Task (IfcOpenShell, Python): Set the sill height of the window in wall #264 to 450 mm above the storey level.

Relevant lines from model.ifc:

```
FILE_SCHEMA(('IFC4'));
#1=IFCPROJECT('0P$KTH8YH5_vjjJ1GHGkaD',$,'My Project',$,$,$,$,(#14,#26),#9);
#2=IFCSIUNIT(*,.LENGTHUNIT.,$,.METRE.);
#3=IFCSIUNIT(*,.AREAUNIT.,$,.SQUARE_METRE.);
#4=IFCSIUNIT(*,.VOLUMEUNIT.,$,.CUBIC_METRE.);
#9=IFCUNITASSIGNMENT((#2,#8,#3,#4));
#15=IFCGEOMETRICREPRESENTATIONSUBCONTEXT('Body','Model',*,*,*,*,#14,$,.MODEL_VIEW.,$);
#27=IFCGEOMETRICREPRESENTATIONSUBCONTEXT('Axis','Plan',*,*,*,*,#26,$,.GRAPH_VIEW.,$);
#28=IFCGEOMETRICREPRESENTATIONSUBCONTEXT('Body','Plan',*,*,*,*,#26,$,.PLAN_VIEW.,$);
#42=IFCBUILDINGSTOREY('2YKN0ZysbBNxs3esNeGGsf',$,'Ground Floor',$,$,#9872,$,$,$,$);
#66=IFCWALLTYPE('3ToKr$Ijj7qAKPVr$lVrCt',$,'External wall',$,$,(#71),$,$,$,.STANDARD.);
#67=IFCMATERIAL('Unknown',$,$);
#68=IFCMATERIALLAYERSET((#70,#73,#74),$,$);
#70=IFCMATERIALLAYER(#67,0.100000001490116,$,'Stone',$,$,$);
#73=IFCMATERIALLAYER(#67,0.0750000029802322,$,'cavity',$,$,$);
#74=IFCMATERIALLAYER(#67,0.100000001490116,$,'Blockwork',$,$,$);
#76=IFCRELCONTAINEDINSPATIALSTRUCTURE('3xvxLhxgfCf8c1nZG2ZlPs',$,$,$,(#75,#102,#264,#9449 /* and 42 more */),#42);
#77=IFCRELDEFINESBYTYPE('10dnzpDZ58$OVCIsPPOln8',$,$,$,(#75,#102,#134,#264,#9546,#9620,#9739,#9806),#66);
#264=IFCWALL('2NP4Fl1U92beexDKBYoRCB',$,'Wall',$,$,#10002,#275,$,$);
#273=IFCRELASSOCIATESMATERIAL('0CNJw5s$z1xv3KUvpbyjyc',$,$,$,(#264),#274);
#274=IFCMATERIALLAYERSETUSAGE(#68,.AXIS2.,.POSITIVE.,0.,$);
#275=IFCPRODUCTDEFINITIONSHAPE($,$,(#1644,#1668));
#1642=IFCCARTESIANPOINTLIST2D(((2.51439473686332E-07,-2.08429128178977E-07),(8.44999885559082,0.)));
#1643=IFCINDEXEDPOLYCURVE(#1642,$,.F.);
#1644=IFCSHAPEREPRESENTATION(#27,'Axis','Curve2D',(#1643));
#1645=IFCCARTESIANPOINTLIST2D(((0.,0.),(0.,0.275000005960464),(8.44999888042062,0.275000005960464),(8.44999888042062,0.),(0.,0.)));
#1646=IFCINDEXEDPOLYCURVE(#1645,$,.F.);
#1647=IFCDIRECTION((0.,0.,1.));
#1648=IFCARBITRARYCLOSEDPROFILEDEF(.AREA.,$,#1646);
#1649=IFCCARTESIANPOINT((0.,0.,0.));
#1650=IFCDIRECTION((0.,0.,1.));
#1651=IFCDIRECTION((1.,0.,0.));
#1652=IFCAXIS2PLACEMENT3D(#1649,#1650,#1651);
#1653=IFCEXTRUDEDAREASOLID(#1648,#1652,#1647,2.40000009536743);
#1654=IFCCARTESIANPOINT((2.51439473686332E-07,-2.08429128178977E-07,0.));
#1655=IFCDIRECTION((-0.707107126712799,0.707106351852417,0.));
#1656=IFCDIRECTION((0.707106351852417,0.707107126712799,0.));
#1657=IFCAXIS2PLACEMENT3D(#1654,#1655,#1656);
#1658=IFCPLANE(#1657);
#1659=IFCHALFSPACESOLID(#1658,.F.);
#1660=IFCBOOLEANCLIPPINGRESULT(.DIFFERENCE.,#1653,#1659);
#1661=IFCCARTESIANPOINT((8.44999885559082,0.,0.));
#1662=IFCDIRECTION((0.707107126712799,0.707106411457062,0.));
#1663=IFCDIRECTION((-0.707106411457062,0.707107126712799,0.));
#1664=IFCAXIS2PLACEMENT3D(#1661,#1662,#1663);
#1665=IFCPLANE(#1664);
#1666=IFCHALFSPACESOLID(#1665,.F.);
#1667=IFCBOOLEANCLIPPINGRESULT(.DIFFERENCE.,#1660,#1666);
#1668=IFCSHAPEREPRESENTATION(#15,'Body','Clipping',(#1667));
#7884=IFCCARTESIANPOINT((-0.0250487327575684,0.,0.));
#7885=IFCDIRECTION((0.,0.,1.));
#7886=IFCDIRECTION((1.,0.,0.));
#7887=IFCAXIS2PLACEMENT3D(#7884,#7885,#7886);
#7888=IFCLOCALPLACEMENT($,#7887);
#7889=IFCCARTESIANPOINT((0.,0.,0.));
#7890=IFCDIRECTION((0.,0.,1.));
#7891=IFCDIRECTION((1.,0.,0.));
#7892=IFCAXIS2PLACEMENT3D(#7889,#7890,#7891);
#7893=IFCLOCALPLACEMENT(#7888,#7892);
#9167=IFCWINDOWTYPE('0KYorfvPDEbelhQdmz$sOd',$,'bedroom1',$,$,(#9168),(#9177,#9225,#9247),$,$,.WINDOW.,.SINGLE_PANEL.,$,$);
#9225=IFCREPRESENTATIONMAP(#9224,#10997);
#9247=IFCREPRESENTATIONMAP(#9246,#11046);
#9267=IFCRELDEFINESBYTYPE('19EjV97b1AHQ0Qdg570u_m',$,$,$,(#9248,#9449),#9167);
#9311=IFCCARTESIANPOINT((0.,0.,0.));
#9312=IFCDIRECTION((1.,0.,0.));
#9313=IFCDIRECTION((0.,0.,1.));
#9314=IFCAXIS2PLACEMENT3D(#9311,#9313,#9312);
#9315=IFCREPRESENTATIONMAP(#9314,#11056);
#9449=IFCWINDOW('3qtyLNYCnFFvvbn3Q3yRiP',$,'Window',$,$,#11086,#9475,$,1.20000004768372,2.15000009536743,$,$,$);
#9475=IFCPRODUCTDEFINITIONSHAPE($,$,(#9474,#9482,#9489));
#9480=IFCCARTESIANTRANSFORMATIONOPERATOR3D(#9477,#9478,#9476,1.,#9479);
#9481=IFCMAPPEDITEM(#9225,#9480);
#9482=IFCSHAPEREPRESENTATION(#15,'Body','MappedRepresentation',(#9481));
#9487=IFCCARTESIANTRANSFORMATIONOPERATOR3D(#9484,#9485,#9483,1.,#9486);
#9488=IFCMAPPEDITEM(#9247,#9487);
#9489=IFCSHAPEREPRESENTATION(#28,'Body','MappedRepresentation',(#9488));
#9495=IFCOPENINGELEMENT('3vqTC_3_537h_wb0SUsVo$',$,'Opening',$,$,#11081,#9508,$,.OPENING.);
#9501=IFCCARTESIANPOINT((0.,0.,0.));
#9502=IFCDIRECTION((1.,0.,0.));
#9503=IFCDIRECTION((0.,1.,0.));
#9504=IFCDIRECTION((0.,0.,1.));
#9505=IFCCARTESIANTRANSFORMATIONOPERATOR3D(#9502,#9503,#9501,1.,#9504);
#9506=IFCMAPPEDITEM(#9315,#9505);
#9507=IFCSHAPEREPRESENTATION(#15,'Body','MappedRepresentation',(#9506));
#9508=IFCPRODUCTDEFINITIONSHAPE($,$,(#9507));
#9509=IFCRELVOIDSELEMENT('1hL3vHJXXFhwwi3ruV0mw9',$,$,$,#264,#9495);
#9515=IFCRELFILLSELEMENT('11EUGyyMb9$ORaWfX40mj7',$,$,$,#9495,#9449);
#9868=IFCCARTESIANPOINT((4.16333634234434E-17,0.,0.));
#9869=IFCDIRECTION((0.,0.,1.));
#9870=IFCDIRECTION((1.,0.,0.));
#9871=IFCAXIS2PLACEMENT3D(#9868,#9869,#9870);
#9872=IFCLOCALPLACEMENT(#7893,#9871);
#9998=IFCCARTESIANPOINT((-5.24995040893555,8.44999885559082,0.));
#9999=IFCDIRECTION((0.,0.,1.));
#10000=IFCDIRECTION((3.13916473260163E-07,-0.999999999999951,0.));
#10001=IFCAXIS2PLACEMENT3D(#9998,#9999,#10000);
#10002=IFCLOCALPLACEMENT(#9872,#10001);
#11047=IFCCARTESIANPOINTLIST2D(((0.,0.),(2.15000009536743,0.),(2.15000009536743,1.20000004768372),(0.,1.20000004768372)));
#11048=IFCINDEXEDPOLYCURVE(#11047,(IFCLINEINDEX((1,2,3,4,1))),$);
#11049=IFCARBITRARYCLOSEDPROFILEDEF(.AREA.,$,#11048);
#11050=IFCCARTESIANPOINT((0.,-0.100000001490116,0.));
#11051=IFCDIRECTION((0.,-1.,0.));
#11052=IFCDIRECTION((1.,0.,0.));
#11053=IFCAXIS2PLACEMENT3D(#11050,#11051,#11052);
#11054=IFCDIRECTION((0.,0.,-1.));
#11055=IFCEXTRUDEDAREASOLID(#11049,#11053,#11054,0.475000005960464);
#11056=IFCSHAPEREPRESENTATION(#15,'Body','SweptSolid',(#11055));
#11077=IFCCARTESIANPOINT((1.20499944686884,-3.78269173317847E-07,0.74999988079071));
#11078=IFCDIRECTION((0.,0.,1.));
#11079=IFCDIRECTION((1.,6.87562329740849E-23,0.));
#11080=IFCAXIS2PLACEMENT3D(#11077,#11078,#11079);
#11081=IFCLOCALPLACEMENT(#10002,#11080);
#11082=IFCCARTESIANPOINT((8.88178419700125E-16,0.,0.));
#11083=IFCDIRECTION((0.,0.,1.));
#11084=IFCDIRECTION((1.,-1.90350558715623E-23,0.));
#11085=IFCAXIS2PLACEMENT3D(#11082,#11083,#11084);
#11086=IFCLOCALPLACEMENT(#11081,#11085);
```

```python
import numpy as np
import ifcopenshell
import ifcopenshell.api.geometry
import ifcopenshell.geom
import ifcopenshell.util.element
import ifcopenshell.util.placement
import ifcopenshell.util.shape
import ifcopenshell.util.unit

model = ifcopenshell.open("model.ifc")
unit_scale = ifcopenshell.util.unit.calculate_unit_scale(model)

window = model.by_guid("3qtyLNYCnFFvvbn3Q3yRiP")
opening = window.FillsVoids[0].RelatingOpeningElement
storey = ifcopenshell.util.element.get_container(window, ifc_class="IfcBuildingStorey")
level = ifcopenshell.util.placement.get_local_placement(storey.ObjectPlacement)[2, 3]

# The opening's origin need not be at the sill, so measure its lowest point.
shape = ifcopenshell.geom.create_shape(ifcopenshell.geom.settings(), opening)
bottom = ifcopenshell.util.shape.get_shape_bottom_elevation(shape, shape.geometry) / unit_scale
dz = level + 0.45 / unit_scale - bottom

shift = np.array([0.0, 0.0, dz])
# The window is placed relative to its opening, so it follows when the opening moves.
matrix = ifcopenshell.util.placement.get_local_placement(opening.ObjectPlacement)
matrix[:3, 3] += shift
ifcopenshell.api.geometry.edit_object_placement(
    model, product=opening, matrix=matrix, is_si=False, should_transform_children=True
)

print(f"moved by {dz * unit_scale:+.3f} m")

model.write("model-out.ifc")
```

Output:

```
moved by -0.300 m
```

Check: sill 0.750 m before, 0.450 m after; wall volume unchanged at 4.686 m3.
